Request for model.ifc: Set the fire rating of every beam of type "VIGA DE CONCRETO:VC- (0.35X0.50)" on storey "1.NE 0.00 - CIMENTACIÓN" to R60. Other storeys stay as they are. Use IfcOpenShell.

First a look at what the model holds.

```python
import ifcopenshell
import ifcopenshell.util.element

model = ifcopenshell.open("model.ifc")
print(model.schema)
storey = next(s for s in model.by_type("IfcBuildingStorey") if s.Name == "1.NE 0.00 - CIMENTACIÓN")
beams = [e for e in ifcopenshell.util.element.get_decomposition(storey) if e.is_a("IfcBeam")]
seen = {}
for e in beams:
    element_type = ifcopenshell.util.element.get_type(e)
    key = (element_type.Name if element_type != e and element_type else None, ifcopenshell.util.element.get_pset(e, "Pset_BeamCommon", "FireRating"))
    seen[key] = seen.get(key, 0) + 1
for (name, value), count in sorted(seen.items(), key=str):
    print(count, "x", name, "|", value)
```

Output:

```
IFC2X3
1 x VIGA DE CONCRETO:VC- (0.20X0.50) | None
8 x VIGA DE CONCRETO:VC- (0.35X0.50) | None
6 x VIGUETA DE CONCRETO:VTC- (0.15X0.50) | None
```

```python
import ifcopenshell
import ifcopenshell.api.pset
import ifcopenshell.util.element

model = ifcopenshell.open("model.ifc")

storey = next(s for s in model.by_type("IfcBuildingStorey") if s.Name == "1.NE 0.00 - CIMENTACIÓN")
beams = [e for e in ifcopenshell.util.element.get_decomposition(storey) if e.is_a("IfcBeam")]

count = 0
for e in beams:
    element_type = ifcopenshell.util.element.get_type(e)
    if element_type in (None, e) or element_type.Name != "VIGA DE CONCRETO:VC- (0.35X0.50)":
        continue
    # add_pset returns the element's existing set when there is one.
    pset = ifcopenshell.api.pset.add_pset(model, product=e, name="Pset_BeamCommon")
    ifcopenshell.api.pset.edit_pset(model, pset=pset, properties={"FireRating": "R60"})
    count += 1

print(count, "beams updated")

model.write("model_v2.ifc")
```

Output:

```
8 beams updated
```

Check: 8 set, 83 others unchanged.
